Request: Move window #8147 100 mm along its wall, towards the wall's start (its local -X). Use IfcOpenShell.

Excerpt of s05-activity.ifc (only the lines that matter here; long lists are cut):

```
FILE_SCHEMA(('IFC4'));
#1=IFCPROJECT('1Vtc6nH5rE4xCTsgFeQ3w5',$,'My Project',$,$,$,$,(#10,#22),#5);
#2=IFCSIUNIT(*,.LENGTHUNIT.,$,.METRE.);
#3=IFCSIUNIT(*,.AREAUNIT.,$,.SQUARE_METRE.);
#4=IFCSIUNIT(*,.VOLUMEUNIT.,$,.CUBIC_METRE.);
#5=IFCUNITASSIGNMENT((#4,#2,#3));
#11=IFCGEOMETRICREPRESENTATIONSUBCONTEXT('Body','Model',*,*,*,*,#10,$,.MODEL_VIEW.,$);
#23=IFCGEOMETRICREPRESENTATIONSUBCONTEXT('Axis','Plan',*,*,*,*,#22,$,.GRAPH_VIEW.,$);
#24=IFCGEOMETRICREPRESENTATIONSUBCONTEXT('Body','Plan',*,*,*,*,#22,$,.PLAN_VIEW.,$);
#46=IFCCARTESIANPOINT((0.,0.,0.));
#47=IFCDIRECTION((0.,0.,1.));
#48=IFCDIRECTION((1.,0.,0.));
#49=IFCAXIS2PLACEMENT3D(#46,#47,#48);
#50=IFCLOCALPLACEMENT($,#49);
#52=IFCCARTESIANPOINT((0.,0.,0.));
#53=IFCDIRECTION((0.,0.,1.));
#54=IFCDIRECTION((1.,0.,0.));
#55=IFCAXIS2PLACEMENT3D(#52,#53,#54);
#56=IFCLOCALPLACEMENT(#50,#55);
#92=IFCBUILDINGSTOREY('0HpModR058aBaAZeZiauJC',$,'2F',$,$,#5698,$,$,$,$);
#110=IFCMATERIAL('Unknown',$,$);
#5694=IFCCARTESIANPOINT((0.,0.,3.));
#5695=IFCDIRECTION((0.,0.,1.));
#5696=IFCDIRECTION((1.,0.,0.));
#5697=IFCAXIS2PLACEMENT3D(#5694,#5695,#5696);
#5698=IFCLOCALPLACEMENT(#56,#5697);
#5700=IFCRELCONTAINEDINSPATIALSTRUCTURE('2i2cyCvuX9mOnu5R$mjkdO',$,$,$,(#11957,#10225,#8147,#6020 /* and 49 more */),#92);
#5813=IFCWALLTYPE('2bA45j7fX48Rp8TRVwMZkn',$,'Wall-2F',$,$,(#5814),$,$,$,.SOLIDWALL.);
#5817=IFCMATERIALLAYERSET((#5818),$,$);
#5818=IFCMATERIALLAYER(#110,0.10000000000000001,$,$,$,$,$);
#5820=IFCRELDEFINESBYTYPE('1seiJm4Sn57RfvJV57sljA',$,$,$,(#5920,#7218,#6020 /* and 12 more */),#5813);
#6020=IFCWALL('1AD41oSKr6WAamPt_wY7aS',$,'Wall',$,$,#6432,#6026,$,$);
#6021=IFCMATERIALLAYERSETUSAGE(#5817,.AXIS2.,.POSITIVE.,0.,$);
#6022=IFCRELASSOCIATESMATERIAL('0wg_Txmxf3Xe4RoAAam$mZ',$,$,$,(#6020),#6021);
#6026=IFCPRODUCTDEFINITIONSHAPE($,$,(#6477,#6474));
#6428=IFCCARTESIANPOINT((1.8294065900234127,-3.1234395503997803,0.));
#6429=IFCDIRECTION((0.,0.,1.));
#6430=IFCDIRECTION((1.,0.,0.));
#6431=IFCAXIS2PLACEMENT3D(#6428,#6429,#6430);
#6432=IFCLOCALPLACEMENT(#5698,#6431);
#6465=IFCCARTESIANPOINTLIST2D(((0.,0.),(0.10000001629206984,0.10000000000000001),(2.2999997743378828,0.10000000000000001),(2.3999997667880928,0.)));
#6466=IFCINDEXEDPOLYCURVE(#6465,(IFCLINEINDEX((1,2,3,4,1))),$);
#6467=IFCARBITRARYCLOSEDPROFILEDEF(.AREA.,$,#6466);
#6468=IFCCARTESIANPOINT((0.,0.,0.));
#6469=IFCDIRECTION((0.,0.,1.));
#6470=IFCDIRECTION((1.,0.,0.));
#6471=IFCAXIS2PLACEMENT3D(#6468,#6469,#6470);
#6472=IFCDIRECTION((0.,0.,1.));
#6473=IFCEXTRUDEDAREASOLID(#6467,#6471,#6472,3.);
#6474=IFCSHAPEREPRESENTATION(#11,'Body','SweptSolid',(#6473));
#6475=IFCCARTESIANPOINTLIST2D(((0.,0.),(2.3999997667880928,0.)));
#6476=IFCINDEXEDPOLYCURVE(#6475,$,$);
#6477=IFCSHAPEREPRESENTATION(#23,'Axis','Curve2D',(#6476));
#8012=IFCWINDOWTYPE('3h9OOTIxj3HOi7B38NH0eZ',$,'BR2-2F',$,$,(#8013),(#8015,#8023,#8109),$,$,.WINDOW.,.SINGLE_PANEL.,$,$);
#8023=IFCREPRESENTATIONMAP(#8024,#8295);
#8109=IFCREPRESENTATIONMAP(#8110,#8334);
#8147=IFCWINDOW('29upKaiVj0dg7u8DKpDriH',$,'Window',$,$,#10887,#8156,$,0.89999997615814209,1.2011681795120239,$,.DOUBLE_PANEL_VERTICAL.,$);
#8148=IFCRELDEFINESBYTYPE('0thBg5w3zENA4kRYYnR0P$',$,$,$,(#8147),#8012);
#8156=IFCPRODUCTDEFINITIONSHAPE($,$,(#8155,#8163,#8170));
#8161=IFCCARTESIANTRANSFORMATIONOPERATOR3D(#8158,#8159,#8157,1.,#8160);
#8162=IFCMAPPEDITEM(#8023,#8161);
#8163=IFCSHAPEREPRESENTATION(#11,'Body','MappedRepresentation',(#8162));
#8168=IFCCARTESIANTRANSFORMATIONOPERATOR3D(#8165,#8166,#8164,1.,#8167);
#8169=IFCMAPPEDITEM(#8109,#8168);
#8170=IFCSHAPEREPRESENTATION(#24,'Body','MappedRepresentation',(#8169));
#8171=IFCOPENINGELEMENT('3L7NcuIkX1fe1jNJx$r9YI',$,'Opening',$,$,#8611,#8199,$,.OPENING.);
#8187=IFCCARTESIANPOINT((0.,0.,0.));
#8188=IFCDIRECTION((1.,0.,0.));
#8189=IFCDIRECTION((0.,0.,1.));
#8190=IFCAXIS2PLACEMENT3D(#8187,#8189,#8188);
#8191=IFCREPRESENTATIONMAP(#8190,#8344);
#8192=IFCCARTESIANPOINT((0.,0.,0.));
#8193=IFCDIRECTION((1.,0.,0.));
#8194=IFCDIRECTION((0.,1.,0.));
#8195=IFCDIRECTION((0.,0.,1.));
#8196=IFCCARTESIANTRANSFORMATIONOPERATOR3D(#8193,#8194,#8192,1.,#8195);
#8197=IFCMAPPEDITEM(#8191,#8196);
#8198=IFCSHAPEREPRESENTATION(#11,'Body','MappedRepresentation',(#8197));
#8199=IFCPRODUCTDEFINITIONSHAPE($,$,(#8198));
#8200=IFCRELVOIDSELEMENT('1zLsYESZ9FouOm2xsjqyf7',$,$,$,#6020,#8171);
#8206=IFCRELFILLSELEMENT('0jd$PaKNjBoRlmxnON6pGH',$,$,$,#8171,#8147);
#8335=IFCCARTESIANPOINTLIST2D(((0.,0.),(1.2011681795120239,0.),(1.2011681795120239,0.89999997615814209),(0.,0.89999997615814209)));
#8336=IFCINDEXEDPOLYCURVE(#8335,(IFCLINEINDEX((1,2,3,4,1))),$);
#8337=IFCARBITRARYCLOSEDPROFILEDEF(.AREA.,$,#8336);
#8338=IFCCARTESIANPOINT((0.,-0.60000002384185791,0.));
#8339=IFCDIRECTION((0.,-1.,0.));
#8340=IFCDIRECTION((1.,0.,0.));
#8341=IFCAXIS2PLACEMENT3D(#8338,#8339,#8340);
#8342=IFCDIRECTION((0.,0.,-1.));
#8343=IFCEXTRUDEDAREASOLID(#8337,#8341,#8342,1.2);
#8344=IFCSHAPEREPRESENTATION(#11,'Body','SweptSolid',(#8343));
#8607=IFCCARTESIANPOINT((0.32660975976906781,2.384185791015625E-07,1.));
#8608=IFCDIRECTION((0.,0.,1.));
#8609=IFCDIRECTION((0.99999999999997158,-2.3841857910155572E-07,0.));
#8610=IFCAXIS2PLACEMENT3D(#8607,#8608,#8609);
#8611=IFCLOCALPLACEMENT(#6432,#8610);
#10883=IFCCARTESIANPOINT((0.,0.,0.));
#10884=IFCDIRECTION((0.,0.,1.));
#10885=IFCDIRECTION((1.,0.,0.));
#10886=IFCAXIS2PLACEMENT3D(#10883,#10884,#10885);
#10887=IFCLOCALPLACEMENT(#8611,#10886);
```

```python
import ifcopenshell
import ifcopenshell.api.geometry
import ifcopenshell.util.placement

model = ifcopenshell.open("s05-activity.ifc")

window = model.by_guid("29upKaiVj0dg7u8DKpDriH")
opening = window.FillsVoids[0].RelatingOpeningElement
wall = opening.VoidsElements[0].RelatingBuildingElement

wall_matrix = ifcopenshell.util.placement.get_local_placement(wall.ObjectPlacement)
shift = wall_matrix[:3, 0] * -0.1
before = ifcopenshell.util.placement.get_local_placement(window.ObjectPlacement)[:3, 3].copy()

# The window is placed relative to its opening, so it follows when the opening moves.
matrix = ifcopenshell.util.placement.get_local_placement(opening.ObjectPlacement)
matrix[:3, 3] += shift
ifcopenshell.api.geometry.edit_object_placement(
    model, product=opening, matrix=matrix, is_si=False, should_transform_children=True
)

after = ifcopenshell.util.placement.get_local_placement(window.ObjectPlacement)[:3, 3]
print("window moved by", (after - before).round(3) + 0.0)

model.write("s05-activity-out.ifc")
```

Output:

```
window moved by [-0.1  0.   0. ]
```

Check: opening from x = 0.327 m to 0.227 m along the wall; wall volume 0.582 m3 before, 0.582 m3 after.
